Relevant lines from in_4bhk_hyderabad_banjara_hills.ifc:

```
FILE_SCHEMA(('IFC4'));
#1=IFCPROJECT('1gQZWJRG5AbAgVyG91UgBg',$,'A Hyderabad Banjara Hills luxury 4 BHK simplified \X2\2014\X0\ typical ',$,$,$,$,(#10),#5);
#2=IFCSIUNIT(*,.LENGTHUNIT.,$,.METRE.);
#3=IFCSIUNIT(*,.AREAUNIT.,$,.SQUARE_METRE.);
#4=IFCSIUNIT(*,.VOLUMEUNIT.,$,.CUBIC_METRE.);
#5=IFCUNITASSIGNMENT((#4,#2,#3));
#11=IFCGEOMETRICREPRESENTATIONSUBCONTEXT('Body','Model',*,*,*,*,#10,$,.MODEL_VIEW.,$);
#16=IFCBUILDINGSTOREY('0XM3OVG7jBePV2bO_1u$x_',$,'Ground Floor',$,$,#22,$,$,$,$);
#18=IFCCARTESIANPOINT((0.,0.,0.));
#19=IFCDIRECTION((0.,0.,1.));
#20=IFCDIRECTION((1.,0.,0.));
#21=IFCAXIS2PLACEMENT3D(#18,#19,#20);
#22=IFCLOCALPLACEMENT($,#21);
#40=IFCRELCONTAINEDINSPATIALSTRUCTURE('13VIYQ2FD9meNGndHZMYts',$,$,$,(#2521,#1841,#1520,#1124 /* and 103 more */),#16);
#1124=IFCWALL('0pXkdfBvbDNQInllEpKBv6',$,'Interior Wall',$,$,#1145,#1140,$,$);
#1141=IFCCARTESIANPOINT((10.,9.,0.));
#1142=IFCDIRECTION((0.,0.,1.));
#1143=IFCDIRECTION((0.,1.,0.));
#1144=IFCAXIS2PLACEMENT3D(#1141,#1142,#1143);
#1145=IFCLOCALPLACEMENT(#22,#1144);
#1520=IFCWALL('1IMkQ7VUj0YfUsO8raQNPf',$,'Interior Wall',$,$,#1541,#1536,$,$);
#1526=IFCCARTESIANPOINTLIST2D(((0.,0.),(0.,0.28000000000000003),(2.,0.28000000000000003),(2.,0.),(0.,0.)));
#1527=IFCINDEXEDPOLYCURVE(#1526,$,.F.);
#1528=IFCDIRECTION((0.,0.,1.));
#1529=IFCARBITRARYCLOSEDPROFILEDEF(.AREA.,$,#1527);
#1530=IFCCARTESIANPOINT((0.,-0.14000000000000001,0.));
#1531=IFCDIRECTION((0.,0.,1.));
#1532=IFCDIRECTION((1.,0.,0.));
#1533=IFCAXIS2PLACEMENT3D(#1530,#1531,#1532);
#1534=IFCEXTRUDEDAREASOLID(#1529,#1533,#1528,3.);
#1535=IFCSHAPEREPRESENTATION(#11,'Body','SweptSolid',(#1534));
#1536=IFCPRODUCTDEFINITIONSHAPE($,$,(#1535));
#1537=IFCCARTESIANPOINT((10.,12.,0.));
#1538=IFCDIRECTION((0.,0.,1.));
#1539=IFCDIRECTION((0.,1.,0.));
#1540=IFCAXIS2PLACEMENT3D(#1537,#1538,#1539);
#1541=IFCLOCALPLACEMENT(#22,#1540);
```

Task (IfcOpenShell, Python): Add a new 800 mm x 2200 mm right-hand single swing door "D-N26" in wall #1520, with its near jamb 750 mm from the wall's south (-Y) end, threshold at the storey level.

```python
import numpy as np
import ifcopenshell
import ifcopenshell.api.feature
import ifcopenshell.api.geometry
import ifcopenshell.api.root
import ifcopenshell.api.spatial
import ifcopenshell.geom
import ifcopenshell.util.element
import ifcopenshell.util.placement
import ifcopenshell.util.representation
import ifcopenshell.util.shape
import ifcopenshell.util.unit

model = ifcopenshell.open("in_4bhk_hyderabad_banjara_hills.ifc")
unit_scale = ifcopenshell.util.unit.calculate_unit_scale(model)
settings = ifcopenshell.geom.settings()


def volume(element):
    """Net volume in cubic metres, openings subtracted."""
    shape = ifcopenshell.geom.create_shape(settings, element)
    return ifcopenshell.util.shape.get_volume(shape.geometry)


wall = model.by_guid("1IMkQ7VUj0YfUsO8raQNPf")
storey = ifcopenshell.util.element.get_container(wall, ifc_class="IfcBuildingStorey")
context = ifcopenshell.util.representation.get_context(model, "Model", "Body", "MODEL_VIEW")
before = volume(wall)

width, height, from_end, sill = 0.8, 2.2, 0.75, 0.0  # metres

# The wall runs along its own X axis, and the end named is its -X end.
wall_shape = ifcopenshell.geom.create_shape(settings, wall)
x, y, z = ifcopenshell.util.shape.get_vertices(wall_shape.geometry).T
start = x.min() + from_end
face, thickness = float(y.min()), float(y.max() - y.min())
wall_matrix = ifcopenshell.util.placement.get_local_placement(wall.ObjectPlacement)
level = ifcopenshell.util.placement.get_local_placement(storey.ObjectPlacement)[2, 3]


def in_wall(x, y):
    """Placement at x, y metres in the wall's axes, at sill height."""
    matrix = wall_matrix.copy()
    matrix[:, 3] = wall_matrix @ np.array([x / unit_scale, y / unit_scale, 0.0, 1.0])
    matrix[2, 3] = level + sill / unit_scale
    return matrix


# Opening: a box that overshoots both wall faces by 50 mm.
opening = ifcopenshell.api.root.create_entity(model, ifc_class="IfcOpeningElement", predefined_type="OPENING")
box = ifcopenshell.api.geometry.add_wall_representation(
    model, context=context, length=width, height=height, thickness=thickness + 0.1
)
ifcopenshell.api.geometry.assign_representation(model, product=opening, representation=box)
ifcopenshell.api.geometry.edit_object_placement(model, product=opening, matrix=in_wall(start, face - 0.05), is_si=False)
ifcopenshell.api.feature.add_feature(model, feature=opening, element=wall)

door = ifcopenshell.api.root.create_entity(model, ifc_class="IfcDoor", name="D-N26", predefined_type="DOOR")
door.OverallWidth, door.OverallHeight = width / unit_scale, height / unit_scale
door.OperationType = "SINGLE_SWING_RIGHT"
body = ifcopenshell.api.geometry.add_door_representation(
    model,
    context=context,
    overall_width=door.OverallWidth,
    overall_height=door.OverallHeight,
    operation_type="SINGLE_SWING_RIGHT",
    lining_properties={"LiningDepth": thickness / unit_scale, "ThresholdDepth": thickness / unit_scale},
)
ifcopenshell.api.geometry.assign_representation(model, product=door, representation=body)
ifcopenshell.api.spatial.assign_container(model, products=[door], relating_structure=storey)
ifcopenshell.api.feature.add_filling(model, opening=opening, element=door)

# The lining spans the wall, so the door starts at the wall face.
ifcopenshell.api.geometry.edit_object_placement(model, product=door, matrix=in_wall(start, face), is_si=False)

after = volume(wall)

print(f"wall volume {before:.3f} -> {after:.3f} m3")

model.write("in_4bhk_hyderabad_banjara_hills_updated.ifc")
```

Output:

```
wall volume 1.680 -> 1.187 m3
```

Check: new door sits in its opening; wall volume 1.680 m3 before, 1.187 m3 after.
